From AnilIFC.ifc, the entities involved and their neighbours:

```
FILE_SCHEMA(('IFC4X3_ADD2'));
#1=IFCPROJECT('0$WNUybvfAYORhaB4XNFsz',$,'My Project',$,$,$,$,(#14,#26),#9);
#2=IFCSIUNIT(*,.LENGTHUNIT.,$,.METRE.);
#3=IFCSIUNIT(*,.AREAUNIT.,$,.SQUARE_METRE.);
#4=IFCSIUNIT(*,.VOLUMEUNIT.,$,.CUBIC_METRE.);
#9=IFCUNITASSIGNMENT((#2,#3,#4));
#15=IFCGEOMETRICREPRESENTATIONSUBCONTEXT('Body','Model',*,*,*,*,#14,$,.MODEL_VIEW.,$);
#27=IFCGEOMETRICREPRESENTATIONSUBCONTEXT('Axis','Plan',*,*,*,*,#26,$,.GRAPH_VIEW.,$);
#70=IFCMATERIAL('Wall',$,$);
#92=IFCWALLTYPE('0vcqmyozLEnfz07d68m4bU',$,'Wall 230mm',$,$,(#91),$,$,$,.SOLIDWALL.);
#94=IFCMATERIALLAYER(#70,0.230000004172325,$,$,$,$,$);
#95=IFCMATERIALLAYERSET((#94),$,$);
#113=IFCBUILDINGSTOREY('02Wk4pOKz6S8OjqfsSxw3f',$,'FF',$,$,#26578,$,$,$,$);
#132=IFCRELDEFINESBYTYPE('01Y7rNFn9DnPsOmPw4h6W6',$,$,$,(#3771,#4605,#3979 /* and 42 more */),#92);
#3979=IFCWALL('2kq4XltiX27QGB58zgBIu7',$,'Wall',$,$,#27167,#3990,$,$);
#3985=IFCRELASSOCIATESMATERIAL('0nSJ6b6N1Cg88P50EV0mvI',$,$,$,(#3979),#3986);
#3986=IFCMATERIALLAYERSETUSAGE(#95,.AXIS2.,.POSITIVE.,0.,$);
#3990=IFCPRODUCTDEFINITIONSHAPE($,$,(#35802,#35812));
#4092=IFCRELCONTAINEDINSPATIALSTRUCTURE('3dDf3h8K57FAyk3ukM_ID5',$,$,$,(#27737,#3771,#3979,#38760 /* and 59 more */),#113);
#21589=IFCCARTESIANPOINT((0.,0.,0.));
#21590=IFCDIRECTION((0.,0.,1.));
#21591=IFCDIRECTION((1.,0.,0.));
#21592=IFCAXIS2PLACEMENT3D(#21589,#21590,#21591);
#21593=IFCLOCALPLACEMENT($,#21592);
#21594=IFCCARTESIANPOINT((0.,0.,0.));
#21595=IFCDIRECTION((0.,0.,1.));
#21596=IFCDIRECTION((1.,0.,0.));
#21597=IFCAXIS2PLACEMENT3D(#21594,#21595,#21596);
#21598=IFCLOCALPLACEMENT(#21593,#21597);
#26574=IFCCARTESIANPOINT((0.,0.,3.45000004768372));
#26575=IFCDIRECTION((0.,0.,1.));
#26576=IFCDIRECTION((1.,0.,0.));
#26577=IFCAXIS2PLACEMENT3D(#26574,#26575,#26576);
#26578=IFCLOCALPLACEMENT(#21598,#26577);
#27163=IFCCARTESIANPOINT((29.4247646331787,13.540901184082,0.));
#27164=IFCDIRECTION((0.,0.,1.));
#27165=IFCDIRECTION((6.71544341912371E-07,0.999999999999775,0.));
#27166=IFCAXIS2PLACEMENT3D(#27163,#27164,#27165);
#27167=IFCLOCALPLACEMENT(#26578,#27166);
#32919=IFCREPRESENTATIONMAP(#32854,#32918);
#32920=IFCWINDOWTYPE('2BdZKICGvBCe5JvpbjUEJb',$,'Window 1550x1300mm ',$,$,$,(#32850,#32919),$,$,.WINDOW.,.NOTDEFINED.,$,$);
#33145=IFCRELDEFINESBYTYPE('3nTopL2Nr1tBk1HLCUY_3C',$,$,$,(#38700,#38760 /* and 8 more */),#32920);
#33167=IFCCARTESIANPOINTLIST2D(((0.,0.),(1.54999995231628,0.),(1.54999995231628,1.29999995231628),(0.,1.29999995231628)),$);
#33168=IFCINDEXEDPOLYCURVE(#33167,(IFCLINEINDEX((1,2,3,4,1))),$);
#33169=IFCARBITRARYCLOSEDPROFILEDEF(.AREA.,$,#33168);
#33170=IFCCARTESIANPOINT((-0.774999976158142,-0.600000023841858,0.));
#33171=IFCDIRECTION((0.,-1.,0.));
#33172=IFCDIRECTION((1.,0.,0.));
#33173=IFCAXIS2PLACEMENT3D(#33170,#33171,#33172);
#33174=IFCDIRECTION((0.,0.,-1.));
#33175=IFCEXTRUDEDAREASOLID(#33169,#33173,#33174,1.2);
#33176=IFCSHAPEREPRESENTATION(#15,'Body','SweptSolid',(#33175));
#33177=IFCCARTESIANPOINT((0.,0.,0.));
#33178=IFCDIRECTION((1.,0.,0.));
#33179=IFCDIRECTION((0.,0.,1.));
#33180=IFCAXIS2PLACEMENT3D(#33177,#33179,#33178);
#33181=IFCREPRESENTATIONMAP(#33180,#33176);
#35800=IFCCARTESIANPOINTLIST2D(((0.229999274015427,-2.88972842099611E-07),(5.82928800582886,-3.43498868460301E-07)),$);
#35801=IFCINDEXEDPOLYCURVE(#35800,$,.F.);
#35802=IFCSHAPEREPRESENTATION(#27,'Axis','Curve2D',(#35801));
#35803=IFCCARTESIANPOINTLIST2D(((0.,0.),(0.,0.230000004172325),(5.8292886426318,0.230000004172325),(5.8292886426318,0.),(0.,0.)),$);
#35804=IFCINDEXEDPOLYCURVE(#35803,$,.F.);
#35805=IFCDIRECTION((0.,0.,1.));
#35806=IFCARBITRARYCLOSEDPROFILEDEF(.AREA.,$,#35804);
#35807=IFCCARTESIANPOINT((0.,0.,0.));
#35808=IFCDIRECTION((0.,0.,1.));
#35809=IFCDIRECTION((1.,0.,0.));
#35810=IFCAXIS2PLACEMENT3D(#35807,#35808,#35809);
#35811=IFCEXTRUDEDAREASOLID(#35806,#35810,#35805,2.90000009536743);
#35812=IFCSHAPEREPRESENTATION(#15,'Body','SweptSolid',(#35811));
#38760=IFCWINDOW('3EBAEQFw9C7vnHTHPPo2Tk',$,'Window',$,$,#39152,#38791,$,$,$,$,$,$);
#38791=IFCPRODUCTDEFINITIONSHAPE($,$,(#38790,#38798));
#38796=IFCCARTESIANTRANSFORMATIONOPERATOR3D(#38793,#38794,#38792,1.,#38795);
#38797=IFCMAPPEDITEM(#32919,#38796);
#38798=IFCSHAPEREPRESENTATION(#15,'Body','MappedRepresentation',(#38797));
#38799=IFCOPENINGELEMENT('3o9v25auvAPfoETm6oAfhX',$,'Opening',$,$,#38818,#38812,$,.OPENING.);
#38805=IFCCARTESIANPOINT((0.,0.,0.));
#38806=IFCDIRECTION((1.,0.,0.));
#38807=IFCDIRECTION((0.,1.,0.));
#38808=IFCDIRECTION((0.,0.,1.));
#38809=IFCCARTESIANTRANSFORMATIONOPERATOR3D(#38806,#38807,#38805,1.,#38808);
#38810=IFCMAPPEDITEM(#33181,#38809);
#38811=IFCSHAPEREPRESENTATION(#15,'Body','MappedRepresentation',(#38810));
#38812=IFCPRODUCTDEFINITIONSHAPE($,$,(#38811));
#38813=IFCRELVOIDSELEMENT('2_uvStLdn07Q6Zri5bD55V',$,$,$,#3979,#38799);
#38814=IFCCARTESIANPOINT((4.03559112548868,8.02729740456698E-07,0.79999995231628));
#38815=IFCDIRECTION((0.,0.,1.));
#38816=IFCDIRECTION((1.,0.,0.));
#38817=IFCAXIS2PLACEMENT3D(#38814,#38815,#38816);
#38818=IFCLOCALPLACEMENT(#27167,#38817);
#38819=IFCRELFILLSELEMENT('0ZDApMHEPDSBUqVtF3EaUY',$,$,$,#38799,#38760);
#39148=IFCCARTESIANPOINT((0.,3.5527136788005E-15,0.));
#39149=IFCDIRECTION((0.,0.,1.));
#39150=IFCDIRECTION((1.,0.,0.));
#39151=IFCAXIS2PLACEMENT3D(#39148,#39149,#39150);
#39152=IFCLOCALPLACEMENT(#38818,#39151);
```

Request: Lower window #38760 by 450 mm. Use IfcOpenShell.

```python
import numpy as np
import ifcopenshell
import ifcopenshell.api.geometry
import ifcopenshell.util.placement
import ifcopenshell.util.unit

model = ifcopenshell.open("AnilIFC.ifc")
unit_scale = ifcopenshell.util.unit.calculate_unit_scale(model)

window = model.by_guid("3EBAEQFw9C7vnHTHPPo2Tk")
opening = window.FillsVoids[0].RelatingOpeningElement
dz = -0.45 / unit_scale

shift = np.array([0.0, 0.0, dz])
# The window is placed relative to its opening, so it follows when the opening moves.
matrix = ifcopenshell.util.placement.get_local_placement(opening.ObjectPlacement)
matrix[:3, 3] += shift
ifcopenshell.api.geometry.edit_object_placement(
    model, product=opening, matrix=matrix, is_si=False, should_transform_children=True
)

print(f"moved by {dz * unit_scale:+.3f} m")

model.write("AnilIFC_edited.ifc")
```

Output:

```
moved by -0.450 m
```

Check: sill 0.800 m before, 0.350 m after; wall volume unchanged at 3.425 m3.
